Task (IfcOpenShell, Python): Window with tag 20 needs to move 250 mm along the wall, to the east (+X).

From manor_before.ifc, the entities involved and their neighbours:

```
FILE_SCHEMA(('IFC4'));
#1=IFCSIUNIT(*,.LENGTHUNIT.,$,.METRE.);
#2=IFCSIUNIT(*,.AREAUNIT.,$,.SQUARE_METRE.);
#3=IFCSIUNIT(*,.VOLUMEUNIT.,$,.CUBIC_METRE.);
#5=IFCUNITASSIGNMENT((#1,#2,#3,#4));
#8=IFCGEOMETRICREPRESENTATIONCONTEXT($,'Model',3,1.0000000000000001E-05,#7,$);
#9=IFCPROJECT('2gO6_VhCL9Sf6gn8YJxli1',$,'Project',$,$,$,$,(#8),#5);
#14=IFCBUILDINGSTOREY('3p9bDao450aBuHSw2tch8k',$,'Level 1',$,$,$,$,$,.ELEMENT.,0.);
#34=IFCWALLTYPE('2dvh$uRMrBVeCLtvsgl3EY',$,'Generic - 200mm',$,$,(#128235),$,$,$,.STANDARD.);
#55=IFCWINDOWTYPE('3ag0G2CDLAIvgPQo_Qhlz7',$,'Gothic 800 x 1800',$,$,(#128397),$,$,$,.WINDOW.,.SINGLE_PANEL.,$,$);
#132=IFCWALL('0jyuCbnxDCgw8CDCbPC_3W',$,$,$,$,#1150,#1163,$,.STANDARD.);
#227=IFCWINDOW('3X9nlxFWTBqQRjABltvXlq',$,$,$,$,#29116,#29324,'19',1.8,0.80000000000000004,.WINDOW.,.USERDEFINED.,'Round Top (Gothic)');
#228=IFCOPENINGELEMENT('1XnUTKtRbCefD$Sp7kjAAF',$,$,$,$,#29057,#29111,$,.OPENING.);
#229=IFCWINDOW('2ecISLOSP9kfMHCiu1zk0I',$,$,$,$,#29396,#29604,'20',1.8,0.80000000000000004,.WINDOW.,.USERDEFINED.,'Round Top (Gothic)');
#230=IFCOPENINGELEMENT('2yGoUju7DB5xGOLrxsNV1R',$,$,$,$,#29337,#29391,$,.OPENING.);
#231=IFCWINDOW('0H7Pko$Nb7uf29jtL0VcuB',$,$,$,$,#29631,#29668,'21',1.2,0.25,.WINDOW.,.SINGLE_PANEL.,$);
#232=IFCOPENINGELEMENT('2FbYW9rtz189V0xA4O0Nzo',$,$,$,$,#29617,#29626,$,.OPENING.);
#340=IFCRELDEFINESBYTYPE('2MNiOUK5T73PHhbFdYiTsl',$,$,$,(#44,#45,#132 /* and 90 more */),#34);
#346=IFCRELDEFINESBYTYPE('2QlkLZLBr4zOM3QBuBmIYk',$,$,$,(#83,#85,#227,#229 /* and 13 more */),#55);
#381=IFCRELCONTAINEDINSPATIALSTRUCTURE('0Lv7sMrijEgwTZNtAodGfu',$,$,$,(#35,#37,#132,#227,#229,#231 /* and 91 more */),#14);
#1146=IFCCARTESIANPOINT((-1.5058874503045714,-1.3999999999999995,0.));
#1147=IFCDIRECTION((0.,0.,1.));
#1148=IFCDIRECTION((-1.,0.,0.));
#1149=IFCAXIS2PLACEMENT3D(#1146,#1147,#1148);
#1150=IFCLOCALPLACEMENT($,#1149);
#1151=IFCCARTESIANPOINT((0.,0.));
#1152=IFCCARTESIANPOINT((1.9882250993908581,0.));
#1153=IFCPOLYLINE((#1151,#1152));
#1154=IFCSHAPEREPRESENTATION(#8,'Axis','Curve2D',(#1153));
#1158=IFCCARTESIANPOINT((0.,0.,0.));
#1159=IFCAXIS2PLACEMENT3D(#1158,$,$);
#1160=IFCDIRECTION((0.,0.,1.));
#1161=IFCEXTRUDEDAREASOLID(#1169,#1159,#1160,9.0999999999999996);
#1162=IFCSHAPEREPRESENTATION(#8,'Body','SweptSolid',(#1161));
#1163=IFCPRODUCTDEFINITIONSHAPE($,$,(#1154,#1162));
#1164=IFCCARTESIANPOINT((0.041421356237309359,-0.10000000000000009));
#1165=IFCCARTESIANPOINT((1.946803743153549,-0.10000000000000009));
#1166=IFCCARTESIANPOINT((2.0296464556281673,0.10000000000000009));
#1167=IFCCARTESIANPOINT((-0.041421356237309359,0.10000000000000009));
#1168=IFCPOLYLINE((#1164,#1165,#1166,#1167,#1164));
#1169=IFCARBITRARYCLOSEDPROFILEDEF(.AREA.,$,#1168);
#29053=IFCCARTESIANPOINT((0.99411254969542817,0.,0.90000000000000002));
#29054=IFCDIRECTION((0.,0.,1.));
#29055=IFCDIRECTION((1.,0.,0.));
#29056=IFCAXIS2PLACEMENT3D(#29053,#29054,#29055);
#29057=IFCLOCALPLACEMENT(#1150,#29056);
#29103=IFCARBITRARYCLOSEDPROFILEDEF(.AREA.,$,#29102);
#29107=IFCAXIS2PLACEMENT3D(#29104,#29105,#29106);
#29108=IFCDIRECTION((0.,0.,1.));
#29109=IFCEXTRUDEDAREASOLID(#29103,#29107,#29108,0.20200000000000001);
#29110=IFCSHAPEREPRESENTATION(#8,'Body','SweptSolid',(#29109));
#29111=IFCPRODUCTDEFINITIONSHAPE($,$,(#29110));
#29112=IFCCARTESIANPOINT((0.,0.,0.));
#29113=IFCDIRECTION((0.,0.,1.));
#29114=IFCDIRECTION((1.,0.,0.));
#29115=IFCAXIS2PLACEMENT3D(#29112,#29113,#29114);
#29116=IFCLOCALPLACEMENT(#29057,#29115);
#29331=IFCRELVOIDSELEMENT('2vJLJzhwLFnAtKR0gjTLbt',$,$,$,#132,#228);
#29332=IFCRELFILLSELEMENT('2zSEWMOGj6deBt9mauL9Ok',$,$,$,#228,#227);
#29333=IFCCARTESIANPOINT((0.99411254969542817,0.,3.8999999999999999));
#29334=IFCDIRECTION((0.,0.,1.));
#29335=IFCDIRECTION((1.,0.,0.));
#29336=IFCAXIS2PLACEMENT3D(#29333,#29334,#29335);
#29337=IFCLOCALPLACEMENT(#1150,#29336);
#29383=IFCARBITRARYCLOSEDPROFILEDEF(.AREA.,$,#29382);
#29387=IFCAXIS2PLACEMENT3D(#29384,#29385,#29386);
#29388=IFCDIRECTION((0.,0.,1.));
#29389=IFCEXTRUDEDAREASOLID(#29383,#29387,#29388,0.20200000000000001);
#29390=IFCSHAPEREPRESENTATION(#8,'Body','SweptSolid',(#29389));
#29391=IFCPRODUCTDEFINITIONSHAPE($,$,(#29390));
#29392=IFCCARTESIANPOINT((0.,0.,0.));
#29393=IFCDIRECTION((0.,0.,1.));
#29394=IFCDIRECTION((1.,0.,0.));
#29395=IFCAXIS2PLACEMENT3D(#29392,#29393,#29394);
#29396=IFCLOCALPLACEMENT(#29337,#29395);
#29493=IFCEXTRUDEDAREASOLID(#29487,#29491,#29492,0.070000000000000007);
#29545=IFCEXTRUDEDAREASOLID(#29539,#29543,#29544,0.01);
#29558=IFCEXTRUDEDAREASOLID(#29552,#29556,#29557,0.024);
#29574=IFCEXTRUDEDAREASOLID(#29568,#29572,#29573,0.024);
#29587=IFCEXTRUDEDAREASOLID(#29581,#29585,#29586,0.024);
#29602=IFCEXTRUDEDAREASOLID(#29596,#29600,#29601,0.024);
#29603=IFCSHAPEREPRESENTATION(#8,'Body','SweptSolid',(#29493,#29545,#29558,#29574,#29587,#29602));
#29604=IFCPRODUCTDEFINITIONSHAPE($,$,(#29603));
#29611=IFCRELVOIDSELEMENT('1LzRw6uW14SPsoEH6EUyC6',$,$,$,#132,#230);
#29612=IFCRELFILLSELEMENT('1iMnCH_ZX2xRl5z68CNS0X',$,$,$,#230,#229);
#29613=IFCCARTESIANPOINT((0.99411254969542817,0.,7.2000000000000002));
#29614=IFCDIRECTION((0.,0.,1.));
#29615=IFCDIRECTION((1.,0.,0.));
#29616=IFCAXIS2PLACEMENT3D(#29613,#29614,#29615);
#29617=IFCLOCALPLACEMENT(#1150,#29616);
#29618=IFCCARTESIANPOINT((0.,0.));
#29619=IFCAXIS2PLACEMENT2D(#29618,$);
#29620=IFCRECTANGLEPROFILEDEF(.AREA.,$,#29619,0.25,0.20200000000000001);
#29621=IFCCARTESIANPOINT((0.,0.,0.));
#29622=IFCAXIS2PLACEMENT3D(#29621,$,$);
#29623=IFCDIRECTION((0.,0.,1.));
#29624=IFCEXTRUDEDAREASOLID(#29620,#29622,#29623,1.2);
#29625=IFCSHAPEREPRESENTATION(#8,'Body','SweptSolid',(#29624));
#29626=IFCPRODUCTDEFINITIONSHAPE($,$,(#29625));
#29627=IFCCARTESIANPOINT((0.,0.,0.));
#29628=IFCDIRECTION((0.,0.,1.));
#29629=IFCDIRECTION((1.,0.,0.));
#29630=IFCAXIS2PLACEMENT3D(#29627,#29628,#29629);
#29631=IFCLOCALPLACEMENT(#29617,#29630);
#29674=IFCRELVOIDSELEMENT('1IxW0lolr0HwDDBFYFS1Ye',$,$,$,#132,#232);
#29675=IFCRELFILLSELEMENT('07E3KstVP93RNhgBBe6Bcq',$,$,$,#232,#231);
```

```python
import ifcopenshell
import ifcopenshell.api.geometry
import ifcopenshell.util.placement

model = ifcopenshell.open("manor_before.ifc")

window = model.by_guid("2ecISLOSP9kfMHCiu1zk0I")
opening = window.FillsVoids[0].RelatingOpeningElement
wall = opening.VoidsElements[0].RelatingBuildingElement

wall_matrix = ifcopenshell.util.placement.get_local_placement(wall.ObjectPlacement)
shift = wall_matrix[:3, 0] * -0.25
before = ifcopenshell.util.placement.get_local_placement(window.ObjectPlacement)[:3, 3].copy()

# The window is placed relative to its opening, so it follows when the opening moves.
matrix = ifcopenshell.util.placement.get_local_placement(opening.ObjectPlacement)
matrix[:3, 3] += shift
ifcopenshell.api.geometry.edit_object_placement(
    model, product=opening, matrix=matrix, is_si=False, should_transform_children=True
)

after = ifcopenshell.util.placement.get_local_placement(window.ObjectPlacement)[:3, 3]
print("window moved by", (after - before).round(3) + 0.0)

model.write("manor_before_v2.ifc")
```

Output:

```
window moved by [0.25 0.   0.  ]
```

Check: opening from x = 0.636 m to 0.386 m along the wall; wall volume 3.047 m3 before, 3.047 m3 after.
